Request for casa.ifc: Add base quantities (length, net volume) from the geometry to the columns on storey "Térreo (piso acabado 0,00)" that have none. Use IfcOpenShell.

First a look at what the model holds.

```python
import ifcopenshell
import ifcopenshell.util.element
import ifcopenshell.util.unit

model = ifcopenshell.open("casa.ifc")
print(model.schema)
for unit_type in ("LENGTHUNIT", "AREAUNIT", "VOLUMEUNIT"):
    print(unit_type, ifcopenshell.util.unit.calculate_unit_scale(model, unit_type))
storey = next(s for s in model.by_type("IfcBuildingStorey") if s.Name == "Térreo (piso acabado 0,00)")
columns = [e for e in ifcopenshell.util.element.get_decomposition(storey) if e.is_a("IfcColumn")]
for e in sorted(columns, key=lambda e: e.id()):
    print(e.id(), e.is_a(), e.Name, list(ifcopenshell.util.element.get_psets(e, qtos_only=True)), sep=" | ")
```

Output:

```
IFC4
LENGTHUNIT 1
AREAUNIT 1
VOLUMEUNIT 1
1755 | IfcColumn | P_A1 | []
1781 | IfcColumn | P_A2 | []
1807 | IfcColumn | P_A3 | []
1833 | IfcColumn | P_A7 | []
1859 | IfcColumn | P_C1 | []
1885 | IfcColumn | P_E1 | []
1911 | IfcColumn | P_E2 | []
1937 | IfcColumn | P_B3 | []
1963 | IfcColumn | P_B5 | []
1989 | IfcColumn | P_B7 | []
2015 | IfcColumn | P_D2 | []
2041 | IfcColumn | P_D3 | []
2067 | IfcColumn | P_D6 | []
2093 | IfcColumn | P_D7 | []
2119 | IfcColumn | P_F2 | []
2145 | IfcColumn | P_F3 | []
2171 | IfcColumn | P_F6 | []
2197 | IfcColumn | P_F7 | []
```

```python
import ifcopenshell
import ifcopenshell.api.pset
import ifcopenshell.geom
import ifcopenshell.util.element
import ifcopenshell.util.shape
import ifcopenshell.util.unit

model = ifcopenshell.open("casa.ifc")
unit_scale = ifcopenshell.util.unit.calculate_unit_scale(model)
volume_scale = ifcopenshell.util.unit.calculate_unit_scale(model, "VOLUMEUNIT")
settings = ifcopenshell.geom.settings()

storey = next(s for s in model.by_type("IfcBuildingStorey") if s.Name == "Térreo (piso acabado 0,00)")
columns = [e for e in ifcopenshell.util.element.get_decomposition(storey) if e.is_a("IfcColumn")]

for e in sorted(columns, key=lambda e: e.id()):
    if ifcopenshell.util.element.get_psets(e, qtos_only=True, should_inherit=False):
        continue
    # Geometry comes back in metres, in the element's own axes.
    shape = ifcopenshell.geom.create_shape(settings, e)
    values = {
        "Length": ifcopenshell.util.shape.get_z(shape.geometry) / unit_scale,
        "NetVolume": ifcopenshell.util.shape.get_volume(shape.geometry) / volume_scale,
    }
    qto = ifcopenshell.api.pset.add_qto(model, product=e, name="Qto_ColumnBaseQuantities")
    ifcopenshell.api.pset.edit_qto(model, qto=qto, properties=values)
    print(e.id(), {k: round(v, 3) for k, v in values.items()})

model.write("casa_v2.ifc")
```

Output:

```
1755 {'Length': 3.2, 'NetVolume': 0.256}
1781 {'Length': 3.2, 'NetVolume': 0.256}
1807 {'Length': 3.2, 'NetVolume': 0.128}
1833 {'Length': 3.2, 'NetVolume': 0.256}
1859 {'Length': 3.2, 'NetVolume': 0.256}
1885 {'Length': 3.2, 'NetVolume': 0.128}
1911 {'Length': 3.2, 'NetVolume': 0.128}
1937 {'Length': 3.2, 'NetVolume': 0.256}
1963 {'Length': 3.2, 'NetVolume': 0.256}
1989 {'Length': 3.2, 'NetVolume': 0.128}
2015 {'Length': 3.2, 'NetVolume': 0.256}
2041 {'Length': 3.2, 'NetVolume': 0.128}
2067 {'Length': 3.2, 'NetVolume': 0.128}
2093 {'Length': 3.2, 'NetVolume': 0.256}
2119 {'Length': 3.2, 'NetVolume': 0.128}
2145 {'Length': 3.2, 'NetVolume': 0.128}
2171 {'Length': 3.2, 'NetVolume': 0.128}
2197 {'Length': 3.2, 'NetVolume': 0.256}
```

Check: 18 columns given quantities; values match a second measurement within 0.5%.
